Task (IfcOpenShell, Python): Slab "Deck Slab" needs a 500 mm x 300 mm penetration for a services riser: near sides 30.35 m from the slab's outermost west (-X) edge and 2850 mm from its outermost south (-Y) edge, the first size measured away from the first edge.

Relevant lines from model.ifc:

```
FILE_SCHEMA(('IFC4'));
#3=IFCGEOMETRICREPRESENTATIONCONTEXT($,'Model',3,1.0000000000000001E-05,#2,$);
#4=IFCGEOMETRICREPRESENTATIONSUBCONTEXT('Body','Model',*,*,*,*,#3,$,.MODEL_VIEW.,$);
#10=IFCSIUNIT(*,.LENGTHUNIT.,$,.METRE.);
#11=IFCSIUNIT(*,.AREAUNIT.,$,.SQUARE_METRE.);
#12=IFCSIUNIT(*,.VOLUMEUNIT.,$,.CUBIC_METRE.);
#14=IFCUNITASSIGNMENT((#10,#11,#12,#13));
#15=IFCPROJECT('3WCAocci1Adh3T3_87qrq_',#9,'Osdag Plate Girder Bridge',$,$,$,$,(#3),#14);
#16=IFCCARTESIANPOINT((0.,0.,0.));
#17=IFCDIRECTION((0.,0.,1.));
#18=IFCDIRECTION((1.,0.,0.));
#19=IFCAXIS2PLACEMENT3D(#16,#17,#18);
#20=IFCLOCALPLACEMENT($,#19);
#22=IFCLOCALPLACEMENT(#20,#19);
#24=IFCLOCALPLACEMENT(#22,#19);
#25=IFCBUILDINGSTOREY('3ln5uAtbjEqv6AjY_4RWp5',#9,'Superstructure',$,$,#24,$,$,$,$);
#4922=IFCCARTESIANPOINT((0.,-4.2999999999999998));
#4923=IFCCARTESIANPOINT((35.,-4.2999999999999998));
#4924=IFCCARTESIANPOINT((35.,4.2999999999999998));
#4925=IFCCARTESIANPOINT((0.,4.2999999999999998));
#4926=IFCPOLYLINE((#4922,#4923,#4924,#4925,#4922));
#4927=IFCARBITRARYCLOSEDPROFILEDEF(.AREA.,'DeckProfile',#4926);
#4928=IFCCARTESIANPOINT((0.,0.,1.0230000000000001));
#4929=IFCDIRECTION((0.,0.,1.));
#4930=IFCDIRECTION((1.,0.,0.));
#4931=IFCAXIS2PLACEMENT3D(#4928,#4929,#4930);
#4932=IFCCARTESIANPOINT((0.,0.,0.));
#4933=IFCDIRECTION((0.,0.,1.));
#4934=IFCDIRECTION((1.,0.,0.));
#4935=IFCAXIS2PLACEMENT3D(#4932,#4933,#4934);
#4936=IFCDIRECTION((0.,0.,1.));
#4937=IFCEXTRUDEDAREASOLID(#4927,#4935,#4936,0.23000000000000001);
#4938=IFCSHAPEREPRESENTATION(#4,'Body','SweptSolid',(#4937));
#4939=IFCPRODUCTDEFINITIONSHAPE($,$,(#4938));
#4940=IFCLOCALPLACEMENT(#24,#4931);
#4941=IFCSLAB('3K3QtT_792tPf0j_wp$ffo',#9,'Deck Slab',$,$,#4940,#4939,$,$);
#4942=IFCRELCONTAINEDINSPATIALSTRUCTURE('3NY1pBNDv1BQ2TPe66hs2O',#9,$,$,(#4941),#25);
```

```python
import numpy as np
import ifcopenshell
import ifcopenshell.api.feature
import ifcopenshell.api.geometry
import ifcopenshell.api.root
import ifcopenshell.geom
import ifcopenshell.util.placement
import ifcopenshell.util.representation
import ifcopenshell.util.shape
import ifcopenshell.util.unit

model = ifcopenshell.open("model.ifc")
unit_scale = ifcopenshell.util.unit.calculate_unit_scale(model)
settings = ifcopenshell.geom.settings()


def volume(element):
    """Net volume in cubic metres, openings subtracted."""
    shape = ifcopenshell.geom.create_shape(settings, element)
    return ifcopenshell.util.shape.get_volume(shape.geometry)


slab = model.by_guid("3K3QtT_792tPf0j_wp$ffo")
before = volume(slab)

# Extent in the slab's own axes, in metres. The edges named are its -X and -Y sides.
slab_shape = ifcopenshell.geom.create_shape(settings, slab)
vertices = ifcopenshell.util.shape.get_vertices(slab_shape.geometry)
x_min, y_min, bottom = vertices.min(axis=0)
top = vertices[:, 2].max()

opening = ifcopenshell.api.root.create_entity(model, ifc_class="IfcOpeningElement", name="Services riser opening", predefined_type="OPENING")
context = ifcopenshell.util.representation.get_context(model, "Model", "Body", "MODEL_VIEW")
width, depth = 0.5, 0.3
outline = [(0.0, 0.0), (width, 0.0), (width, depth), (0.0, depth), (0.0, 0.0)]
# Overshoot both faces by 50 mm so the cut is clean.
shape = ifcopenshell.api.geometry.add_slab_representation(
    model, context=context, depth=top - bottom + 0.1, polyline=outline
)
ifcopenshell.api.geometry.assign_representation(model, product=opening, representation=shape)

matrix = ifcopenshell.util.placement.get_local_placement(slab.ObjectPlacement)
matrix[:, 3] = matrix @ np.append(np.array([x_min + 30.35, y_min + 2.85, bottom - 0.05]) / unit_scale, 1.0)
ifcopenshell.api.geometry.edit_object_placement(model, product=opening, matrix=matrix, is_si=False)
ifcopenshell.api.feature.add_feature(model, feature=opening, element=slab)

after = volume(slab)

print(f"slab volume {before:.3f} -> {after:.3f} m3")

model.write("model_rev.ifc")
```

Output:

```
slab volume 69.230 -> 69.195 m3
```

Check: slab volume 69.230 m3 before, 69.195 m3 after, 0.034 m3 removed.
